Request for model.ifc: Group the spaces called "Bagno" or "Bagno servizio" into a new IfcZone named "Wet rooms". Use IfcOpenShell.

First a look at what the model holds.

```python
import ifcopenshell

model = ifcopenshell.open("model.ifc")
print(model.schema)
seen = {}
for space in model.by_type("IfcSpace"):
    seen[space.LongName] = seen.get(space.LongName, 0) + 1
for name, count in sorted(seen.items(), key=str):
    print(count, "x", name)
print("zones:", [z.Name for z in model.by_type("IfcZone")][:20])
```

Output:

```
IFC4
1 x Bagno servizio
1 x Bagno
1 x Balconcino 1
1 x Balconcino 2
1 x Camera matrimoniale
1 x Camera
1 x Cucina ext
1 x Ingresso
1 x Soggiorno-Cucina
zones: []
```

```python
import ifcopenshell
import ifcopenshell.api.group
import ifcopenshell.api.root

model = ifcopenshell.open("model.ifc")

names = {"Bagno", "Bagno servizio"}
spaces = [s for s in model.by_type("IfcSpace") if s.LongName in names]

zone = ifcopenshell.api.root.create_entity(model, ifc_class="IfcZone", name="Wet rooms")
ifcopenshell.api.group.assign_group(model, products=spaces, group=zone)
print(len(spaces), "spaces in", zone.Name)

model.write("model-out.ifc")
```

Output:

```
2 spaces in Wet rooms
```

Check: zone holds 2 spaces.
